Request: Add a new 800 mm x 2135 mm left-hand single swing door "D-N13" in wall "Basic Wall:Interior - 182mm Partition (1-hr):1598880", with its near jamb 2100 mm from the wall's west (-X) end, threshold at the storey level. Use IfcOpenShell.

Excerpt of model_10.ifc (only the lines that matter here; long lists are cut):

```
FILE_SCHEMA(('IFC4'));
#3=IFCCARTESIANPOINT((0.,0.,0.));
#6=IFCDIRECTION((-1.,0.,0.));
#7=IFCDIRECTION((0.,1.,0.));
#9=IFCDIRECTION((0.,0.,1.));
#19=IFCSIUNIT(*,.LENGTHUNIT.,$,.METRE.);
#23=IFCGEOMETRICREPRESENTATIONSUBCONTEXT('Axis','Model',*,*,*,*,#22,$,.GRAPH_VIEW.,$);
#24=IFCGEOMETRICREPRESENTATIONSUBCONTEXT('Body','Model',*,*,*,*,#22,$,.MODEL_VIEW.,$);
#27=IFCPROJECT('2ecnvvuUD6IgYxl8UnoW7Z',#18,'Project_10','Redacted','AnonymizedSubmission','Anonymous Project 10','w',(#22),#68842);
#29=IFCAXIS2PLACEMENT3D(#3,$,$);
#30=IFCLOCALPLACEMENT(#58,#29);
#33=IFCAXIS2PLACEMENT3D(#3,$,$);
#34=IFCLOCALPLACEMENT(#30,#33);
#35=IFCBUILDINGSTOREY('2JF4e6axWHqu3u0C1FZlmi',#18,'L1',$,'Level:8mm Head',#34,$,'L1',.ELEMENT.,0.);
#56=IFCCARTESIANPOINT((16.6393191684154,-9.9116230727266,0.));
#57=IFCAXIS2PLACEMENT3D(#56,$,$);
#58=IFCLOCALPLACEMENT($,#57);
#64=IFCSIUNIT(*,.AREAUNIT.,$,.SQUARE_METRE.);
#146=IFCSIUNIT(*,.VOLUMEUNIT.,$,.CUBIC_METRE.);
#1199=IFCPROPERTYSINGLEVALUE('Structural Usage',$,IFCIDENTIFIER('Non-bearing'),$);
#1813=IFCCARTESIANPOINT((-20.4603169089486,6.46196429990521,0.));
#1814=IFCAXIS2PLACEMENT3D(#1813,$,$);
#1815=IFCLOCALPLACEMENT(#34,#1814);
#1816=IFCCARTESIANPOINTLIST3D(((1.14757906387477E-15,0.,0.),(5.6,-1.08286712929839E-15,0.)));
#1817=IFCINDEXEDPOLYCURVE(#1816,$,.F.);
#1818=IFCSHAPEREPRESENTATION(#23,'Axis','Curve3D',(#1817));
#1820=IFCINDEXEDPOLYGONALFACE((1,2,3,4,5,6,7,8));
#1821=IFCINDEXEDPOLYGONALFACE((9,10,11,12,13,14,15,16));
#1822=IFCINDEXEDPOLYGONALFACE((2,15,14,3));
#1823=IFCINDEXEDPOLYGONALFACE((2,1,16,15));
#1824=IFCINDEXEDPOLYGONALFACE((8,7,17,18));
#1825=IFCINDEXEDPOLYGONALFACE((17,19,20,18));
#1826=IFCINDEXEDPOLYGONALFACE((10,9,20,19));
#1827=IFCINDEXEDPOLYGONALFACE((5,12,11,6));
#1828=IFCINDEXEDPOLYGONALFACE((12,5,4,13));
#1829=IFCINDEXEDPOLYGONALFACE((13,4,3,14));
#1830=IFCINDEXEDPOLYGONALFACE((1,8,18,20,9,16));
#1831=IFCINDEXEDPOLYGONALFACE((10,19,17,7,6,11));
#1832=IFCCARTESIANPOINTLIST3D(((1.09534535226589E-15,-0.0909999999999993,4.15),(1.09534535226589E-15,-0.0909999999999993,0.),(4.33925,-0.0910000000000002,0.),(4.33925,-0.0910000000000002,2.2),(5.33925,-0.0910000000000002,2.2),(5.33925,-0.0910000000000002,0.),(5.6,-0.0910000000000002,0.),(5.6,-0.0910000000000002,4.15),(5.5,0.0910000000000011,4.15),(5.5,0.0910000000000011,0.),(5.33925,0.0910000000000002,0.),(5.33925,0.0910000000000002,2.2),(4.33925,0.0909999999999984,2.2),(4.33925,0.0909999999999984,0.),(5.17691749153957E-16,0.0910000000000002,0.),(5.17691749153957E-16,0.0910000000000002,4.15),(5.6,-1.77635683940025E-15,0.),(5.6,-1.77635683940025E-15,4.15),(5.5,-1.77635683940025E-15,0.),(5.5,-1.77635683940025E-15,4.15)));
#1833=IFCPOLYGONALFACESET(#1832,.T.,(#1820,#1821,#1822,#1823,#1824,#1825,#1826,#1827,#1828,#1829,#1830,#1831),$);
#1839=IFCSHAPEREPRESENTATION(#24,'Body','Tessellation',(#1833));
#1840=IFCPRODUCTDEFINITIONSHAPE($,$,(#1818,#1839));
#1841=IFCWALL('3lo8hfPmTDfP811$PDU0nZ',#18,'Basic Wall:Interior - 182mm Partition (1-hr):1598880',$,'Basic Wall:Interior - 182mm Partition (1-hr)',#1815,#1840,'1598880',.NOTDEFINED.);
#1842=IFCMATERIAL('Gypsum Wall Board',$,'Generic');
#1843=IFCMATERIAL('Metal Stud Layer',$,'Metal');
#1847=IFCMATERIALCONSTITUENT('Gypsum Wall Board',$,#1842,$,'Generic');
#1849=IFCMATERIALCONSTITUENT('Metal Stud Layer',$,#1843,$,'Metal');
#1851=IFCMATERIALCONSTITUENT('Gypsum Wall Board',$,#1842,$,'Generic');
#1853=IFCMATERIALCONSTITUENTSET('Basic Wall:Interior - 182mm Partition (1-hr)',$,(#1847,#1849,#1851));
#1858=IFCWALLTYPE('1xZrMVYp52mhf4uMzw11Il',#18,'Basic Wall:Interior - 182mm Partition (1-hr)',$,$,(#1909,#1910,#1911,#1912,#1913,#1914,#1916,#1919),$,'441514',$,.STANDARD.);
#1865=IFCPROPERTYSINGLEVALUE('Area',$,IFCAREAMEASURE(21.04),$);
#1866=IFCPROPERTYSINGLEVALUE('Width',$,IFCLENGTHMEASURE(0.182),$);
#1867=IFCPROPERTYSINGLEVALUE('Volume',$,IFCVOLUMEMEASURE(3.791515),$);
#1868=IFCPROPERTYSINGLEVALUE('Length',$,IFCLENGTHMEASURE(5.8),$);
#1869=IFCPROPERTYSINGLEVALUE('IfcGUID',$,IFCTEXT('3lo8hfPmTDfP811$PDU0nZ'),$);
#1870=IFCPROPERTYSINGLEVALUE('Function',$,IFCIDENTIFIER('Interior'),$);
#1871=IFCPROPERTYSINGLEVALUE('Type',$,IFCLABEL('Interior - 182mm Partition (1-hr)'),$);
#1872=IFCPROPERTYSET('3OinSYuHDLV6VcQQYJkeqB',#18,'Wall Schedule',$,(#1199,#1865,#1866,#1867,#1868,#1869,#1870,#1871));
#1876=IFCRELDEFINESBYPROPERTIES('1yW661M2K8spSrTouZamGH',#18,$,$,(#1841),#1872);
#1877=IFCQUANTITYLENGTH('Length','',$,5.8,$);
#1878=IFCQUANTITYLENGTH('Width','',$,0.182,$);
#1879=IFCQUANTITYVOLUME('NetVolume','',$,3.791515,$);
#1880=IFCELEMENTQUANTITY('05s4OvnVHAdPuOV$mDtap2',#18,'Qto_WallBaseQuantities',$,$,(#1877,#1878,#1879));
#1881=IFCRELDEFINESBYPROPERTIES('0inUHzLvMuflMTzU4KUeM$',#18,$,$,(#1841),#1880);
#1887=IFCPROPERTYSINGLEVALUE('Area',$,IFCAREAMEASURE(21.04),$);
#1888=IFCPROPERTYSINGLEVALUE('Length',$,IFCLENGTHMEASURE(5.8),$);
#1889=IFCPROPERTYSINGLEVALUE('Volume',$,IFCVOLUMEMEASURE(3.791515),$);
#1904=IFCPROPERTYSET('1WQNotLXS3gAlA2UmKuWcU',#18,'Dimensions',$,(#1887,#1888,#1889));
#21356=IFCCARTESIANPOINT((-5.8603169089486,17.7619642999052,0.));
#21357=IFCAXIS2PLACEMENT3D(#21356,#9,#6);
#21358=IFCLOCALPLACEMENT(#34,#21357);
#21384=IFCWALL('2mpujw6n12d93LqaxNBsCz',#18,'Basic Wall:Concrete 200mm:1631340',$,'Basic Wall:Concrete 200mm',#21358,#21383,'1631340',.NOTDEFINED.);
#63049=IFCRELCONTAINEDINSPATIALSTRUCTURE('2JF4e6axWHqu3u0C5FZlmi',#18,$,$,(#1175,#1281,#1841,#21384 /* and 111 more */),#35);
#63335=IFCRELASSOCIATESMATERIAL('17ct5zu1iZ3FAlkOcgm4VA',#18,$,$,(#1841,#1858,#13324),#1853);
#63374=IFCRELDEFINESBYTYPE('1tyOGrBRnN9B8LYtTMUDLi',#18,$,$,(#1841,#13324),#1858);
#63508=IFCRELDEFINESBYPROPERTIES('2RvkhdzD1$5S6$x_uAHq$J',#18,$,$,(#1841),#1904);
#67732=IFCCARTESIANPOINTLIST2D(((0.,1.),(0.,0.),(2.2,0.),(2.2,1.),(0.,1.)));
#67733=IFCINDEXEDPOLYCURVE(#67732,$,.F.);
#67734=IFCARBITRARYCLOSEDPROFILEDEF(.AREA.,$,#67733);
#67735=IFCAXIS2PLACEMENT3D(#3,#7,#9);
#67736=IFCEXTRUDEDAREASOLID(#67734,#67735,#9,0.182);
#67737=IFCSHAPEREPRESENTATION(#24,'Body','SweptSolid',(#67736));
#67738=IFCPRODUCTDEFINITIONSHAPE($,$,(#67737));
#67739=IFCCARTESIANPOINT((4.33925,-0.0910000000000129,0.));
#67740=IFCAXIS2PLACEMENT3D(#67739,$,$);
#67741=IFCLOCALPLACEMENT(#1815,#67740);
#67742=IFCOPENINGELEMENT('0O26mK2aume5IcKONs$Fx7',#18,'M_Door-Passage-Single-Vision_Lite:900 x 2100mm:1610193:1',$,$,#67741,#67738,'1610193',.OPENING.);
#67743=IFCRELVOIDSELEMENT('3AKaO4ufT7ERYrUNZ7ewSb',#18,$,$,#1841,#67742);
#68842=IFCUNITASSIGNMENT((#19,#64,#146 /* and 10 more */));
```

```python
import numpy as np
import ifcopenshell
import ifcopenshell.api.feature
import ifcopenshell.api.geometry
import ifcopenshell.api.pset
import ifcopenshell.api.root
import ifcopenshell.api.spatial
import ifcopenshell.geom
import ifcopenshell.util.element
import ifcopenshell.util.placement
import ifcopenshell.util.representation
import ifcopenshell.util.shape
import ifcopenshell.util.unit

model = ifcopenshell.open("model_10.ifc")
unit_scale = ifcopenshell.util.unit.calculate_unit_scale(model)
area_scale = ifcopenshell.util.unit.calculate_unit_scale(model, "AREAUNIT")
volume_scale = ifcopenshell.util.unit.calculate_unit_scale(model, "VOLUMEUNIT")
settings = ifcopenshell.geom.settings()


def volume(element):
    """Net volume in cubic metres, openings subtracted."""
    shape = ifcopenshell.geom.create_shape(settings, element)
    return ifcopenshell.util.shape.get_volume(shape.geometry)


wall = model.by_guid("3lo8hfPmTDfP811$PDU0nZ")
storey = ifcopenshell.util.element.get_container(wall, ifc_class="IfcBuildingStorey")
context = ifcopenshell.util.representation.get_context(model, "Model", "Body", "MODEL_VIEW")
before = volume(wall)

width, height, from_end, sill = 0.8, 2.135, 2.1, 0.0  # metres

# The wall runs along its own X axis, and the end named is its -X end.
wall_shape = ifcopenshell.geom.create_shape(settings, wall)
x, y, z = ifcopenshell.util.shape.get_vertices(wall_shape.geometry).T
start = x.min() + from_end
face, thickness = float(y.min()), float(y.max() - y.min())
wall_matrix = ifcopenshell.util.placement.get_local_placement(wall.ObjectPlacement)
level = ifcopenshell.util.placement.get_local_placement(storey.ObjectPlacement)[2, 3]


def in_wall(x, y):
    """Placement at x, y metres in the wall's axes, at sill height."""
    matrix = wall_matrix.copy()
    matrix[:, 3] = wall_matrix @ np.array([x / unit_scale, y / unit_scale, 0.0, 1.0])
    matrix[2, 3] = level + sill / unit_scale
    return matrix


# Opening: a box that overshoots both wall faces by 50 mm.
opening = ifcopenshell.api.root.create_entity(model, ifc_class="IfcOpeningElement", predefined_type="OPENING")
box = ifcopenshell.api.geometry.add_wall_representation(
    model, context=context, length=width, height=height, thickness=thickness + 0.1
)
ifcopenshell.api.geometry.assign_representation(model, product=opening, representation=box)
ifcopenshell.api.geometry.edit_object_placement(model, product=opening, matrix=in_wall(start, face - 0.05), is_si=False)
ifcopenshell.api.feature.add_feature(model, feature=opening, element=wall)

door = ifcopenshell.api.root.create_entity(model, ifc_class="IfcDoor", name="D-N13", predefined_type="DOOR")
door.OverallWidth, door.OverallHeight = width / unit_scale, height / unit_scale
door.OperationType = "SINGLE_SWING_LEFT"
body = ifcopenshell.api.geometry.add_door_representation(
    model,
    context=context,
    overall_width=door.OverallWidth,
    overall_height=door.OverallHeight,
    operation_type="SINGLE_SWING_LEFT",
    lining_properties={"LiningDepth": thickness / unit_scale, "ThresholdDepth": thickness / unit_scale},
)
ifcopenshell.api.geometry.assign_representation(model, product=door, representation=body)
ifcopenshell.api.spatial.assign_container(model, products=[door], relating_structure=storey)
ifcopenshell.api.feature.add_filling(model, opening=opening, element=door)

# The lining spans the wall, so the door starts at the wall face.
ifcopenshell.api.geometry.edit_object_placement(model, product=door, matrix=in_wall(start, face), is_si=False)

after = volume(wall)

# Update the wall's stored quantities.
pset = model.by_id(ifcopenshell.util.element.get_pset(wall, "Wall Schedule", should_inherit=False)["id"])
ifcopenshell.api.pset.edit_pset(model, pset=pset, properties={
    "Area": model.create_entity("IfcAreaMeasure", after / thickness / area_scale),
    "Volume": model.create_entity("IfcVolumeMeasure", after / volume_scale),
})
qto = model.by_id(ifcopenshell.util.element.get_pset(wall, "Qto_WallBaseQuantities", should_inherit=False)["id"])
ifcopenshell.api.pset.edit_qto(model, qto=qto, properties={"NetVolume": after / volume_scale})
pset = model.by_id(ifcopenshell.util.element.get_pset(wall, "Dimensions", should_inherit=False)["id"])
ifcopenshell.api.pset.edit_pset(model, pset=pset, properties={
    "Area": model.create_entity("IfcAreaMeasure", after / thickness / area_scale),
    "Volume": model.create_entity("IfcVolumeMeasure", after / volume_scale),
})

print(f"wall volume {before:.3f} -> {after:.3f} m3")

model.write("model_10_v2.ifc")
```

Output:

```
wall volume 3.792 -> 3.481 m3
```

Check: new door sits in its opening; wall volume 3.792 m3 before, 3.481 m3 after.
